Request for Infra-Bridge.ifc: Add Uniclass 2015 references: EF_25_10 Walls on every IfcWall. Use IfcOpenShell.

First a look at what the model holds.

```python
import ifcopenshell

model = ifcopenshell.open("Infra-Bridge.ifc")
print(model.schema)
print("classifications:", [c.Name for c in model.by_type("IfcClassification")])
for ifc_class in ("IfcDoor", "IfcRoof", "IfcStair", "IfcWall", "IfcWindow"):
    print(ifc_class, len(model.by_type(ifc_class)))
```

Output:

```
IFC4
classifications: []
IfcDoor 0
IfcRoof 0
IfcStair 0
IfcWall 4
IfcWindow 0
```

```python
import ifcopenshell
import ifcopenshell.api.classification

model = ifcopenshell.open("Infra-Bridge.ifc")

system = ifcopenshell.api.classification.add_classification(model, classification="Uniclass 2015")

codes = {
    "IfcWall": ("EF_25_10", "Walls"),
}
for ifc_class, (code, name) in codes.items():
    products = model.by_type(ifc_class)
    ifcopenshell.api.classification.add_reference(
        model, products=products, classification=system, identification=code, name=name
    )
    print(code, len(products))

model.write("Infra-Bridge_rev.ifc")
```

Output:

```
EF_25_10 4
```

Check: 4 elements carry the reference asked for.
